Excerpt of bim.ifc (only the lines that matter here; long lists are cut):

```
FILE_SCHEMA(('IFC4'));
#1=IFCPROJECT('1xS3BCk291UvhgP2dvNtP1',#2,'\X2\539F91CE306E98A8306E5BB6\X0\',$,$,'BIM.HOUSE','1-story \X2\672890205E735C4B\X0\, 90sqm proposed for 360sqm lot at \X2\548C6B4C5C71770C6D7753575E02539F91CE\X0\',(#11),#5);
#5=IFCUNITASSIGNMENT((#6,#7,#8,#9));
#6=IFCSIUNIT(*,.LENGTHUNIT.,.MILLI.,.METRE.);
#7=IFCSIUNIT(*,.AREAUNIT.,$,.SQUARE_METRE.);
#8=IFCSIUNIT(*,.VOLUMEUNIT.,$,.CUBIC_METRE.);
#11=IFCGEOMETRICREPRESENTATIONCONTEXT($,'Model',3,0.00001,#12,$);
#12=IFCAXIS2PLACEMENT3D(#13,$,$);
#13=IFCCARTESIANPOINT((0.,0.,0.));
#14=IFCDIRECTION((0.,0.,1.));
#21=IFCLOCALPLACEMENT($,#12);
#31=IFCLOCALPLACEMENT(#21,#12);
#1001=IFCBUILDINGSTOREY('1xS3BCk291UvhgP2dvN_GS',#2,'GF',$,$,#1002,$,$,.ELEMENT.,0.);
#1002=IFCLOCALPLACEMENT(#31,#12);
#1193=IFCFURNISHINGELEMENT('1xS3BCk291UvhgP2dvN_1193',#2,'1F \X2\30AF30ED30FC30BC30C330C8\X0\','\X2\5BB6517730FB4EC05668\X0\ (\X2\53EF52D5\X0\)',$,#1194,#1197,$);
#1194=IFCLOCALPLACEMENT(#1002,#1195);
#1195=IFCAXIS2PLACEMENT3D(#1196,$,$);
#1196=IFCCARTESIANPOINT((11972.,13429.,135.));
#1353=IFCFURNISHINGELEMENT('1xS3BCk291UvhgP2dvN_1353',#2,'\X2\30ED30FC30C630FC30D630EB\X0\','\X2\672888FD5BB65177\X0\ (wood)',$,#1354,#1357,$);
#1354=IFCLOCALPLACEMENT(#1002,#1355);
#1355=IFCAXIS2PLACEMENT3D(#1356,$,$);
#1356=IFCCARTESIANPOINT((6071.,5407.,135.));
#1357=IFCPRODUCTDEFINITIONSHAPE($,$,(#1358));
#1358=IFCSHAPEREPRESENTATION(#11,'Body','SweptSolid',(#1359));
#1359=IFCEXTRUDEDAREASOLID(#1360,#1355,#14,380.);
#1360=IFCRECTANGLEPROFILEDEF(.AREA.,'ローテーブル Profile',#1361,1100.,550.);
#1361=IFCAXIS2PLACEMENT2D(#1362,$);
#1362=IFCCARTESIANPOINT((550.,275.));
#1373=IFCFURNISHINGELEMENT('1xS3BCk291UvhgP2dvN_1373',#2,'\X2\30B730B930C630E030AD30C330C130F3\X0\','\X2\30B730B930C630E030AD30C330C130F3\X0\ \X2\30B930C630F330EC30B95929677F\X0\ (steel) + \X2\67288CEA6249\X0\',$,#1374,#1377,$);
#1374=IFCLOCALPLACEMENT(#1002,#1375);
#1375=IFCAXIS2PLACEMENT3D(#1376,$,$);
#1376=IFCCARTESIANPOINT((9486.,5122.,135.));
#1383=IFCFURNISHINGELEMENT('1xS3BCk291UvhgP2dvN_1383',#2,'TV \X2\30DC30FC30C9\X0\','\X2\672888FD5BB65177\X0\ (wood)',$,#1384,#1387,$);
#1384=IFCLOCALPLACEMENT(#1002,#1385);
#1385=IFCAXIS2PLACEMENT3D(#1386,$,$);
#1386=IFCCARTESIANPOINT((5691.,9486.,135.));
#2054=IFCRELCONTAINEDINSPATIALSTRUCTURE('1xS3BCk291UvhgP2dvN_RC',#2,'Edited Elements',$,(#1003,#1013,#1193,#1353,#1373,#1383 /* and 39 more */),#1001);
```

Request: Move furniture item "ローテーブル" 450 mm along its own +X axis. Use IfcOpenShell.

```python
import ifcopenshell
import ifcopenshell.api.geometry
import ifcopenshell.util.placement
import ifcopenshell.util.unit

model = ifcopenshell.open("bim.ifc")
unit_scale = ifcopenshell.util.unit.calculate_unit_scale(model)

item = model.by_guid("1xS3BCk291UvhgP2dvN_1353")
matrix = ifcopenshell.util.placement.get_local_placement(item.ObjectPlacement)
matrix[:3, 3] += matrix[:3, 0] * 0.45 / unit_scale
ifcopenshell.api.geometry.edit_object_placement(model, product=item, matrix=matrix, is_si=False)

print(ifcopenshell.util.placement.get_local_placement(item.ObjectPlacement).round(3) + 0.0)

model.write("bim_v2.ifc")
```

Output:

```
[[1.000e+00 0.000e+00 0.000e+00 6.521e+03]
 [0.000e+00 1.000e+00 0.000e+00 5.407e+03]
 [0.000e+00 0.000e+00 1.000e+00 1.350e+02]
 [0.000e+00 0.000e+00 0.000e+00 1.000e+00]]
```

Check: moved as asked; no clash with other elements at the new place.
